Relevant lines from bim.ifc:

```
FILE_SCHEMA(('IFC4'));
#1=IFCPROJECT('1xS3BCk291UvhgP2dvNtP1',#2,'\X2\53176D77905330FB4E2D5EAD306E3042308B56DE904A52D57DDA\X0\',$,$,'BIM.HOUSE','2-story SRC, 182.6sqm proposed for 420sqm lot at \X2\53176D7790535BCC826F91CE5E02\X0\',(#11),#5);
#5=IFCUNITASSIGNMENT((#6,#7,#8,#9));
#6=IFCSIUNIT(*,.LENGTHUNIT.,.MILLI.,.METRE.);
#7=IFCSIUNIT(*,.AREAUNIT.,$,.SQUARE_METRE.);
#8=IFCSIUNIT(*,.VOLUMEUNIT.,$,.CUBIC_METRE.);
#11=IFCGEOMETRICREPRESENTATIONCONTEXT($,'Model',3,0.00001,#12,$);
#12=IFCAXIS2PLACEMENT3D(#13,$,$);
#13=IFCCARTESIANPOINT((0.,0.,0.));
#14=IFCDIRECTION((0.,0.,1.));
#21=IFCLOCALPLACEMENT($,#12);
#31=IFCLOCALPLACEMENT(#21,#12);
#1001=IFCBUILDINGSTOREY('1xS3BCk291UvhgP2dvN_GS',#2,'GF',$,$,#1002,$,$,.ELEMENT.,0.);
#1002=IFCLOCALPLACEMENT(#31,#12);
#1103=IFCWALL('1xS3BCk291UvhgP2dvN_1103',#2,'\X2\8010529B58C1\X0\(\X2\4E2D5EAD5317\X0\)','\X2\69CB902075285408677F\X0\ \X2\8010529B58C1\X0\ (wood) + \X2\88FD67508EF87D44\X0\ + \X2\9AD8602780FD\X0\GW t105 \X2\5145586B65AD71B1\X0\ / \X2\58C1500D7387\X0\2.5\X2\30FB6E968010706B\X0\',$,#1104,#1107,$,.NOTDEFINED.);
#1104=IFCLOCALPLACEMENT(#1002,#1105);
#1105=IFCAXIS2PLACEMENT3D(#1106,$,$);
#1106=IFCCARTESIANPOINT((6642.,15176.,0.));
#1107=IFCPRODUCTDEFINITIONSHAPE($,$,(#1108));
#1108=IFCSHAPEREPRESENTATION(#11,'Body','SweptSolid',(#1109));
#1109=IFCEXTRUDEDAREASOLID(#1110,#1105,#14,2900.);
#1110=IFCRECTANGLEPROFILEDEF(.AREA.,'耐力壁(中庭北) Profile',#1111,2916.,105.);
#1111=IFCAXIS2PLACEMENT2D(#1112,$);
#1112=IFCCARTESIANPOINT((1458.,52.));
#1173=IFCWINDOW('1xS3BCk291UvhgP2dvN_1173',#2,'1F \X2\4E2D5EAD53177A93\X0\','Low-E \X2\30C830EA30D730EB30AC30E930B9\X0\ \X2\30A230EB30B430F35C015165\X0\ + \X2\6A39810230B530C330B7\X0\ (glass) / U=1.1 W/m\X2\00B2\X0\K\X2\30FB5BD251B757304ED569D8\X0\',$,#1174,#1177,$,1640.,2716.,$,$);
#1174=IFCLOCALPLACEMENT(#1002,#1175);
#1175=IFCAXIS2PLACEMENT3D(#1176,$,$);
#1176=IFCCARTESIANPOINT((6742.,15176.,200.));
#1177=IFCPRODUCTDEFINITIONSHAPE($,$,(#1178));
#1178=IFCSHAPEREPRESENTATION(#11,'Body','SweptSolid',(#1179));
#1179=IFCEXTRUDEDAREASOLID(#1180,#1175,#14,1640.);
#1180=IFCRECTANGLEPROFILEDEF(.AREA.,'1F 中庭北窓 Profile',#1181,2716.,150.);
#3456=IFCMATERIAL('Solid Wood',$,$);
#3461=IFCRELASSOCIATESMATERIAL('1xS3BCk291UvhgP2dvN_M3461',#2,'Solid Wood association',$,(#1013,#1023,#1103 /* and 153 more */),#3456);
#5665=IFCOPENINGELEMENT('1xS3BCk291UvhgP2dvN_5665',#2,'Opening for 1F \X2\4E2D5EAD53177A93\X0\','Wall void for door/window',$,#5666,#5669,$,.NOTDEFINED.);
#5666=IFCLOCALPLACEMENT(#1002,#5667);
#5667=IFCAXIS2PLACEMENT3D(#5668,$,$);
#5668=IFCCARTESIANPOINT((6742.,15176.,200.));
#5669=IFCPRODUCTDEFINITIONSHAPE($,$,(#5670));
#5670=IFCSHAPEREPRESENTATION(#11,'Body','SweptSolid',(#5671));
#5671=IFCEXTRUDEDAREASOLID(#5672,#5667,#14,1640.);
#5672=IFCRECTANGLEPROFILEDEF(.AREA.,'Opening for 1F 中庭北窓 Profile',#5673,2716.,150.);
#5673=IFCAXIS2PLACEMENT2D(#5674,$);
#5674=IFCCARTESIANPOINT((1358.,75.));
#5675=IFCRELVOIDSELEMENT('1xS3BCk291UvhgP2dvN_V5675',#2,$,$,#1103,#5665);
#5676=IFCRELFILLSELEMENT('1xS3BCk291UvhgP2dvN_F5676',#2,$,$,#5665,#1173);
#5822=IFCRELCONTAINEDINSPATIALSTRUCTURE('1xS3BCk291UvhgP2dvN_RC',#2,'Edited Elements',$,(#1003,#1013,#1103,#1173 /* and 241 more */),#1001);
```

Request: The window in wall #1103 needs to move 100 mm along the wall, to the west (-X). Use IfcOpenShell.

```python
import ifcopenshell
import ifcopenshell.api.geometry
import ifcopenshell.util.placement

model = ifcopenshell.open("bim.ifc")

window = model.by_id(1173)
opening = window.FillsVoids[0].RelatingOpeningElement
wall = opening.VoidsElements[0].RelatingBuildingElement

wall_matrix = ifcopenshell.util.placement.get_local_placement(wall.ObjectPlacement)
shift = wall_matrix[:3, 0] * -100.0
before = ifcopenshell.util.placement.get_local_placement(window.ObjectPlacement)[:3, 3].copy()

# The window is not placed relative to its opening, so move both.
for product in (opening, window):
    matrix = ifcopenshell.util.placement.get_local_placement(product.ObjectPlacement)
    matrix[:3, 3] += shift
    ifcopenshell.api.geometry.edit_object_placement(model, product=product, matrix=matrix, is_si=False)

after = ifcopenshell.util.placement.get_local_placement(window.ObjectPlacement)[:3, 3]
print("window moved by", (after - before).round(3) + 0.0)

model.write("bim_edited.ifc")
```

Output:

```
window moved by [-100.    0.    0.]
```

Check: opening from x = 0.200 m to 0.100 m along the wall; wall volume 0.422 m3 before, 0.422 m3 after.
